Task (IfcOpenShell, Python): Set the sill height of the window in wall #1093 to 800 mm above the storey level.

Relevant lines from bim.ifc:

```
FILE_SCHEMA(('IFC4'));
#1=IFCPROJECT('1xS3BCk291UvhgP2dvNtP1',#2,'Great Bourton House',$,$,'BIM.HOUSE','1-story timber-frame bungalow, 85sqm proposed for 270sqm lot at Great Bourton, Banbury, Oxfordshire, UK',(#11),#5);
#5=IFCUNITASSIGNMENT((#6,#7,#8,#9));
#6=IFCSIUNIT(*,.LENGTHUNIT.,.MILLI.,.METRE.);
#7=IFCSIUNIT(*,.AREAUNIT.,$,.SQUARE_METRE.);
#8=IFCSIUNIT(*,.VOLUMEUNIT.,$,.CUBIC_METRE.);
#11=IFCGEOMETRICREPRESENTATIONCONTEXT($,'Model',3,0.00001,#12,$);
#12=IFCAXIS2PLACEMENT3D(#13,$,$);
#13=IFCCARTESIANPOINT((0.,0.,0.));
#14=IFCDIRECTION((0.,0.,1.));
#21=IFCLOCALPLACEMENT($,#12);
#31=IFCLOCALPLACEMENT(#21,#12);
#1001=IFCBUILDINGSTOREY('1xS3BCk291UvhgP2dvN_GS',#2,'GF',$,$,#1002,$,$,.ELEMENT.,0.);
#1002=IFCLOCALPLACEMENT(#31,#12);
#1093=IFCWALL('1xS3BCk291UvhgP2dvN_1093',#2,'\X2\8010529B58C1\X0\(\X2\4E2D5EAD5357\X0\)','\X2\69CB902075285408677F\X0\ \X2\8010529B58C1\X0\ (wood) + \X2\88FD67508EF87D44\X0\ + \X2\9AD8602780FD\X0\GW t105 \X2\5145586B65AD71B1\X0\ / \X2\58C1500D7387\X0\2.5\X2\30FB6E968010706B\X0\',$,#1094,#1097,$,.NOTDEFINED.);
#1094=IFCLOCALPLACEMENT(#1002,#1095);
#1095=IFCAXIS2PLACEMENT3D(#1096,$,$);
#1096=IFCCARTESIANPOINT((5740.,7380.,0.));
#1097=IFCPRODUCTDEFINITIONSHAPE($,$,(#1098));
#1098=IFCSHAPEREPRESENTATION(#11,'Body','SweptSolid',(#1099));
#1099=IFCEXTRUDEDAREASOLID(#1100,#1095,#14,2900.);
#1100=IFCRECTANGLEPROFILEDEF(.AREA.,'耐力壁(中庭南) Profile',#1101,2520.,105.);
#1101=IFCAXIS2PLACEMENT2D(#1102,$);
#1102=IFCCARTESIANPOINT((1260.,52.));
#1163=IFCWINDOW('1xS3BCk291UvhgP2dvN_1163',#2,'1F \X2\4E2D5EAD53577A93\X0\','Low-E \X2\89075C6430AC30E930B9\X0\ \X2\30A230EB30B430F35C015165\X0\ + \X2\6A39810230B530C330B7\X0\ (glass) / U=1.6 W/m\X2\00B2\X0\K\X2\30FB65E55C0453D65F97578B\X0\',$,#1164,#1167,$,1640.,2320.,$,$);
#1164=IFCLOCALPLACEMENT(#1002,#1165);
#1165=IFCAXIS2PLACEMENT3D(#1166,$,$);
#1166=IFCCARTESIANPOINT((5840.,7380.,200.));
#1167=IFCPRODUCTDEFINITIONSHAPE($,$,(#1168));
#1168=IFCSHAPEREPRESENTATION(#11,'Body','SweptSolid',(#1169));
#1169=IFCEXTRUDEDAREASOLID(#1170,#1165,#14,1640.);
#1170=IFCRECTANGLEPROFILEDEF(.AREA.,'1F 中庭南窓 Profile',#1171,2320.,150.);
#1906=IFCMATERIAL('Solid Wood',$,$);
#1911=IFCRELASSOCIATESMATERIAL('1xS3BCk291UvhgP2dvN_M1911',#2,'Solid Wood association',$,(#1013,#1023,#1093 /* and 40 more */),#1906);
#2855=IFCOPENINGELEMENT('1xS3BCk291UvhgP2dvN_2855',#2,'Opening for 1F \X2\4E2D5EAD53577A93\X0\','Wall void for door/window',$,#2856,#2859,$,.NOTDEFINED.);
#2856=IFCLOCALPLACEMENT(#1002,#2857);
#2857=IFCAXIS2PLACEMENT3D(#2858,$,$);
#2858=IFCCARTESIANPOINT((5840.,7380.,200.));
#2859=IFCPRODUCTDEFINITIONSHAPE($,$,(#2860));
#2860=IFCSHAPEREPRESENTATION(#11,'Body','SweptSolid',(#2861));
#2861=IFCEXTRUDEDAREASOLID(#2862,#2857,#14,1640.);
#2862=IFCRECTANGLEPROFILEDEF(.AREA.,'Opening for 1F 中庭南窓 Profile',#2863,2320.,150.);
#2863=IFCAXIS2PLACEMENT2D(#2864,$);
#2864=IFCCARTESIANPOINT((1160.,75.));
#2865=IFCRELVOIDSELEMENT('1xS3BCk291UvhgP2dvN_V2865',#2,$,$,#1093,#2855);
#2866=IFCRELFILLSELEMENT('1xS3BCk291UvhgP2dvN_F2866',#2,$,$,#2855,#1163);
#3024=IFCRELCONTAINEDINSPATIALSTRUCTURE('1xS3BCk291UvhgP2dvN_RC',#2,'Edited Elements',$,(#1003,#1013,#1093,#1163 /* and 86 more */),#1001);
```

```python
import numpy as np
import ifcopenshell
import ifcopenshell.api.geometry
import ifcopenshell.geom
import ifcopenshell.util.element
import ifcopenshell.util.placement
import ifcopenshell.util.shape
import ifcopenshell.util.unit

model = ifcopenshell.open("bim.ifc")
unit_scale = ifcopenshell.util.unit.calculate_unit_scale(model)

window = model.by_id(1163)
opening = window.FillsVoids[0].RelatingOpeningElement
storey = ifcopenshell.util.element.get_container(window, ifc_class="IfcBuildingStorey")
level = ifcopenshell.util.placement.get_local_placement(storey.ObjectPlacement)[2, 3]

# The opening's origin need not be at the sill, so measure its lowest point.
shape = ifcopenshell.geom.create_shape(ifcopenshell.geom.settings(), opening)
bottom = ifcopenshell.util.shape.get_shape_bottom_elevation(shape, shape.geometry) / unit_scale
dz = level + 0.8 / unit_scale - bottom

shift = np.array([0.0, 0.0, dz])
# The window is not placed relative to its opening, so move both.
for product in (opening, window):
    matrix = ifcopenshell.util.placement.get_local_placement(product.ObjectPlacement)
    matrix[:3, 3] += shift
    ifcopenshell.api.geometry.edit_object_placement(model, product=product, matrix=matrix, is_si=False)

print(f"moved by {dz * unit_scale:+.3f} m")

model.write("bim_rev.ifc")
```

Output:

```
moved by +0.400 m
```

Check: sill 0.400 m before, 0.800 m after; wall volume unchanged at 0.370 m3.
